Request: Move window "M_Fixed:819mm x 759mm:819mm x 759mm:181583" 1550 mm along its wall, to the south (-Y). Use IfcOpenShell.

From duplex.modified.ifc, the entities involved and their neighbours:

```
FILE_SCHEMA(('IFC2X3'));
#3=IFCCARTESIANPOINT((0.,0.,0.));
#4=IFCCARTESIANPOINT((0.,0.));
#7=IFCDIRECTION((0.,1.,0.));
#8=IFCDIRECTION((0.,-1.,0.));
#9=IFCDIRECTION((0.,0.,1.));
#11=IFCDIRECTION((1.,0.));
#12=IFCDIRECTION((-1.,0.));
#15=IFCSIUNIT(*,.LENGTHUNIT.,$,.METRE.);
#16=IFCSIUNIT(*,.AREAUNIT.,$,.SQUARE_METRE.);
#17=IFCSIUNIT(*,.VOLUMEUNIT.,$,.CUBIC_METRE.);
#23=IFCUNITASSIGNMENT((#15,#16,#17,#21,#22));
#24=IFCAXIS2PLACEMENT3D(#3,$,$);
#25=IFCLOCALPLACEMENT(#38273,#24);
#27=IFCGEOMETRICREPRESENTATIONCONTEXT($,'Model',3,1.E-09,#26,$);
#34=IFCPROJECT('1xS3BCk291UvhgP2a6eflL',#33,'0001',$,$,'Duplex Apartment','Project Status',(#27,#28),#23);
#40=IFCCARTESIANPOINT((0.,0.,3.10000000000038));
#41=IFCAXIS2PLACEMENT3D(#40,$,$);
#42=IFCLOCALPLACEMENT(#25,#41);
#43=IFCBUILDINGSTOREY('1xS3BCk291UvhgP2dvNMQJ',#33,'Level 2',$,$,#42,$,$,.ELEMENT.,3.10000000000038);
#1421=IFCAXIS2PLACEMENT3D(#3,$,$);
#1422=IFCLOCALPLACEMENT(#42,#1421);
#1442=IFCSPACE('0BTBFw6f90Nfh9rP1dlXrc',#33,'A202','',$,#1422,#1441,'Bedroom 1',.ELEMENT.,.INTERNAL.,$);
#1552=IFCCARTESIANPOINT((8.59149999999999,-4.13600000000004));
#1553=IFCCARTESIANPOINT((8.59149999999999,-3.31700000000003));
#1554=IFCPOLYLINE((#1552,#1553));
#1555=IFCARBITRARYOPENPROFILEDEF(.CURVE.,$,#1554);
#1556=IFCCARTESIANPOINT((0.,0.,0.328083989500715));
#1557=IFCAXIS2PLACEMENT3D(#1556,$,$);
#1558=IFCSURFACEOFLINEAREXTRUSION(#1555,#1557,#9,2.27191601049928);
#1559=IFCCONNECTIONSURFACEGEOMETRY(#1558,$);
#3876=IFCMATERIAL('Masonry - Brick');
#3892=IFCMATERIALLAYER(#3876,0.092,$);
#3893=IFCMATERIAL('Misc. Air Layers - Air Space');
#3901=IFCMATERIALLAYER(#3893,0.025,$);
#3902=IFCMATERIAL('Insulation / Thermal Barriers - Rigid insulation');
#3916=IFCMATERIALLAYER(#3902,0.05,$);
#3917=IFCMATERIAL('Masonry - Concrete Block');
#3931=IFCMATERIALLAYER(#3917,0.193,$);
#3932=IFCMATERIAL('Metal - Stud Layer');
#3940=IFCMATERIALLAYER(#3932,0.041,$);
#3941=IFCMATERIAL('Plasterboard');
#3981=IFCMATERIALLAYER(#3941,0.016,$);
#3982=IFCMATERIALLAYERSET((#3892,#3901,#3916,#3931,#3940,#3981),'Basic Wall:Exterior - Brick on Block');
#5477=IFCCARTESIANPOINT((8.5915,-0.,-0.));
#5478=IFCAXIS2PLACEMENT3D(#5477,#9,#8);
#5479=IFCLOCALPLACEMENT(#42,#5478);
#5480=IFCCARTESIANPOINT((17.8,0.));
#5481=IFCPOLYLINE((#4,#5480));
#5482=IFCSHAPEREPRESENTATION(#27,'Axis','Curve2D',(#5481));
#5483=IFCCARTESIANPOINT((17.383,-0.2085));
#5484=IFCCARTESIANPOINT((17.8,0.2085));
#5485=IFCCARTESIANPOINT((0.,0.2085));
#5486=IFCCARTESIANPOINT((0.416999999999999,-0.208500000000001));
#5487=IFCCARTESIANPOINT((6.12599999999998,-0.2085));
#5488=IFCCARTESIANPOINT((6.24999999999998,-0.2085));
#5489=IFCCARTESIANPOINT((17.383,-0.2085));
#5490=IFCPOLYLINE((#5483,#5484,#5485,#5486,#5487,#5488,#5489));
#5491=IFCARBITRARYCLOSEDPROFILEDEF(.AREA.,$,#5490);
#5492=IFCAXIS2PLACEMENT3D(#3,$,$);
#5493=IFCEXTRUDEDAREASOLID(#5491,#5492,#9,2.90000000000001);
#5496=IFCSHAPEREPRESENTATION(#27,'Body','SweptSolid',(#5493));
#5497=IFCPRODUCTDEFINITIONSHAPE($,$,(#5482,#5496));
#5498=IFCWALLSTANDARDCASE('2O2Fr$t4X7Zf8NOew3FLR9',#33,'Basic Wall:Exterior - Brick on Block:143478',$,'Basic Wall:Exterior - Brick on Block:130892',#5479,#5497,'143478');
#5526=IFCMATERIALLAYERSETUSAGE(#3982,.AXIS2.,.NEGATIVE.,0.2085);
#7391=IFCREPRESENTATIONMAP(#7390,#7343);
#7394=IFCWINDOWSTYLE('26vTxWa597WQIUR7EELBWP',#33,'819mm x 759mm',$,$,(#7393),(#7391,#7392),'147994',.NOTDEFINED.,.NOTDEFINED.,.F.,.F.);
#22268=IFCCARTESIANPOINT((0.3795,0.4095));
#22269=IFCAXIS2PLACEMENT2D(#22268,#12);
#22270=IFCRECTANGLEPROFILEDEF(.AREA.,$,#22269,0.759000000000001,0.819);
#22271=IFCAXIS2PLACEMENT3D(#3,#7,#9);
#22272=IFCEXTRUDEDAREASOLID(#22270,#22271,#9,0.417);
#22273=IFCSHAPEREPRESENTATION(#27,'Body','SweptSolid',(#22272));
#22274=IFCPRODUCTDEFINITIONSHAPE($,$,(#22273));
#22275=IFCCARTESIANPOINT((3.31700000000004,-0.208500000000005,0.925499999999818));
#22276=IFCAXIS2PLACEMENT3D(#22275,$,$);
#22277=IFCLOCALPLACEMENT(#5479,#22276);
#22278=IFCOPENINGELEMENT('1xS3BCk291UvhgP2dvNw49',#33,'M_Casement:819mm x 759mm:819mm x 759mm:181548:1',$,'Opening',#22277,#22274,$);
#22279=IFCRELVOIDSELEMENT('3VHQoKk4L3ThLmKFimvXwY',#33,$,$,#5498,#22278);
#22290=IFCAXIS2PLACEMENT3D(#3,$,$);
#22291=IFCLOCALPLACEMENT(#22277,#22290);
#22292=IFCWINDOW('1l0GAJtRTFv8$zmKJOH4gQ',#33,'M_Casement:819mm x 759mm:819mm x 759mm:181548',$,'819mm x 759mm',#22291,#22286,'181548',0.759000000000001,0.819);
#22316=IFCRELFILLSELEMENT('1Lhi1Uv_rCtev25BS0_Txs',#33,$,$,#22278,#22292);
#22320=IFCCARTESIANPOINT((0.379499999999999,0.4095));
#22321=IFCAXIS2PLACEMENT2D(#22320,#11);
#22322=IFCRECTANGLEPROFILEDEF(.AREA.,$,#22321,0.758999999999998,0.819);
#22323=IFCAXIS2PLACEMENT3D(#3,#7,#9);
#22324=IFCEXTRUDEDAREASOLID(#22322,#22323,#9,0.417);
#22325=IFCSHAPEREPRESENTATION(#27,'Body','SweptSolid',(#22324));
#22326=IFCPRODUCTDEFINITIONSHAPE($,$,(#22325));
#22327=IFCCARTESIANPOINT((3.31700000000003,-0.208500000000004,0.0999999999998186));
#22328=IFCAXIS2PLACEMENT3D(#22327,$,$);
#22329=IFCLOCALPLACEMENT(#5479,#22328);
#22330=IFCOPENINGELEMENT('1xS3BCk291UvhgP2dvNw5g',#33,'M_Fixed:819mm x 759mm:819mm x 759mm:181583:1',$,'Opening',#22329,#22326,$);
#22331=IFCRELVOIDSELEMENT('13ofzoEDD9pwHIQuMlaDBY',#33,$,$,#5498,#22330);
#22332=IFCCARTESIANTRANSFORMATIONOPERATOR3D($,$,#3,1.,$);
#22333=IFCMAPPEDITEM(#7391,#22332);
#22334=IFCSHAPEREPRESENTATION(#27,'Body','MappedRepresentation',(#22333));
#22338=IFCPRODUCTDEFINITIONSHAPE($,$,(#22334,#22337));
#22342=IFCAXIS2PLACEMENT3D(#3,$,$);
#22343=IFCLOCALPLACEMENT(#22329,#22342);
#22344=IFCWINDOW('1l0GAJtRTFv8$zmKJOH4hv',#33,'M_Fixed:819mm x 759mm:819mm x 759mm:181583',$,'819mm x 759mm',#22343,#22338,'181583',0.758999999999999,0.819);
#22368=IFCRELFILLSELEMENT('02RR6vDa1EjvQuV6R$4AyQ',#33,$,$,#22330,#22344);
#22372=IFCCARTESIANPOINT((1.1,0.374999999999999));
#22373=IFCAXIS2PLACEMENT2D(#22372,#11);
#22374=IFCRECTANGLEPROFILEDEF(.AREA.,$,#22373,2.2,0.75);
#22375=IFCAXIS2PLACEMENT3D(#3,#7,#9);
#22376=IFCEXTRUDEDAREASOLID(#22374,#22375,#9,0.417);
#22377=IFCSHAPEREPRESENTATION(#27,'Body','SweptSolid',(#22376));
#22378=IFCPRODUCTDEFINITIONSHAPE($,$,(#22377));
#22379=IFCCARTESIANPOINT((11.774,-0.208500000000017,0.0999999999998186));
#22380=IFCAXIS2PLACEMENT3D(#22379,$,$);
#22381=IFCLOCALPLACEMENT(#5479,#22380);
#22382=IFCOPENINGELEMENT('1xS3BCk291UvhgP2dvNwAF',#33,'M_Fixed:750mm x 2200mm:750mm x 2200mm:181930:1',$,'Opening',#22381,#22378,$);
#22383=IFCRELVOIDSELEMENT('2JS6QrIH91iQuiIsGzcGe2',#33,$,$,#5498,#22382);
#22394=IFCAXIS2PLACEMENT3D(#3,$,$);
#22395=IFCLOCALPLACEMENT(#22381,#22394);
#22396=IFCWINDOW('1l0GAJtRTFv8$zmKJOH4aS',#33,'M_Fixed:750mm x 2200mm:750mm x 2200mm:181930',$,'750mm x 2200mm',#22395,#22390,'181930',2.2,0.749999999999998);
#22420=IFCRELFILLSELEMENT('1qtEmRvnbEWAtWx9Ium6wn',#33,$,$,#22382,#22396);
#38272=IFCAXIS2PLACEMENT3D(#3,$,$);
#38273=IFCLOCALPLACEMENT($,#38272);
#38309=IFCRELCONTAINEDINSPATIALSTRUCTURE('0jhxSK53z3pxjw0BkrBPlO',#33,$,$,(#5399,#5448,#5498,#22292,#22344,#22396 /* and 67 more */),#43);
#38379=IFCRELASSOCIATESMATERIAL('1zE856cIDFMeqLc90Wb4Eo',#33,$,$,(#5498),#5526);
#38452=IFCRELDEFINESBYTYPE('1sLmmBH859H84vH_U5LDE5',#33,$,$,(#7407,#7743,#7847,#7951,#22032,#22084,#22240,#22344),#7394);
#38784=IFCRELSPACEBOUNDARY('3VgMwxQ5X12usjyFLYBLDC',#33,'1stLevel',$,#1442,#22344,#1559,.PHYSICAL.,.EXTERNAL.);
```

```python
import numpy as np
import ifcopenshell
import ifcopenshell.api.geometry
import ifcopenshell.util.placement
import ifcopenshell.util.unit

model = ifcopenshell.open("duplex.modified.ifc")
unit_scale = ifcopenshell.util.unit.calculate_unit_scale(model)

window = model.by_guid("1l0GAJtRTFv8$zmKJOH4hv")
opening = window.FillsVoids[0].RelatingOpeningElement
wall = opening.VoidsElements[0].RelatingBuildingElement

wall_matrix = ifcopenshell.util.placement.get_local_placement(wall.ObjectPlacement)
shift = wall_matrix[:3, 0] * 1.55 / unit_scale
before = ifcopenshell.util.placement.get_local_placement(window.ObjectPlacement)[:3, 3].copy()

# The window is placed relative to its opening, so it follows when the opening moves.
matrix = ifcopenshell.util.placement.get_local_placement(opening.ObjectPlacement)
matrix[:3, 3] += shift
ifcopenshell.api.geometry.edit_object_placement(
    model, product=opening, matrix=matrix, is_si=False, should_transform_children=True
)

# Space boundary surfaces are stored in each space's coordinates; move them too.
for rel in window.ProvidesBoundaries:
    if not rel.ConnectionGeometry:
        continue
    surface = rel.ConnectionGeometry.SurfaceOnRelatingElement
    space_matrix = ifcopenshell.util.placement.get_local_placement(rel.RelatingSpace.ObjectPlacement)
    point = np.array(surface.Position.Location.Coordinates) + space_matrix[:3, :3].T @ shift
    surface.Position = model.createIfcAxis2Placement3D(
        model.createIfcCartesianPoint(point.tolist()), surface.Position.Axis, surface.Position.RefDirection
    )

after = ifcopenshell.util.placement.get_local_placement(window.ObjectPlacement)[:3, 3]
print("window moved by", (after - before).round(3) + 0.0)

model.write("duplex.modified_updated.ifc")
```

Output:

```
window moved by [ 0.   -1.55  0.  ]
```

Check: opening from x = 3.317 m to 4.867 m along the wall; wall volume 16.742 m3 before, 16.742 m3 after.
